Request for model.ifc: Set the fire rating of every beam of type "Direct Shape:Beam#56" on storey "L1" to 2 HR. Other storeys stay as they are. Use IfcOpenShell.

First a look at what the model holds.

```python
import ifcopenshell
import ifcopenshell.util.element

model = ifcopenshell.open("model.ifc")
print(model.schema)
storey = next(s for s in model.by_type("IfcBuildingStorey") if s.Name == "L1")
beams = [e for e in ifcopenshell.util.element.get_decomposition(storey) if e.is_a("IfcBeam")]
seen = {}
for e in beams:
    element_type = ifcopenshell.util.element.get_type(e)
    key = (element_type.Name if element_type != e and element_type else None, ifcopenshell.util.element.get_pset(e, "Pset_BeamCommon", "FireRating"))
    seen[key] = seen.get(key, 0) + 1
for (name, value), count in sorted(seen.items(), key=str):
    print(count, "x", name, "|", value)
```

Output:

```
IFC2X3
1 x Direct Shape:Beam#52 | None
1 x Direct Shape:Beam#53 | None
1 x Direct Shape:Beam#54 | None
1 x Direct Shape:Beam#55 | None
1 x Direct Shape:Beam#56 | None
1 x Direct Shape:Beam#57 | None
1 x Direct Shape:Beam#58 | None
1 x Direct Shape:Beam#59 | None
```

```python
import ifcopenshell
import ifcopenshell.api.pset
import ifcopenshell.util.element

model = ifcopenshell.open("model.ifc")

storey = next(s for s in model.by_type("IfcBuildingStorey") if s.Name == "L1")
beams = [e for e in ifcopenshell.util.element.get_decomposition(storey) if e.is_a("IfcBeam")]

count = 0
for e in beams:
    element_type = ifcopenshell.util.element.get_type(e)
    if element_type in (None, e) or element_type.Name != "Direct Shape:Beam#56":
        continue
    # add_pset returns the element's existing set when there is one.
    pset = ifcopenshell.api.pset.add_pset(model, product=e, name="Pset_BeamCommon")
    ifcopenshell.api.pset.edit_pset(model, pset=pset, properties={"FireRating": "2 HR"})
    count += 1

print(count, "beams updated")

model.write("model_rev.ifc")
```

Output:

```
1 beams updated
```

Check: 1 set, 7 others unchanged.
